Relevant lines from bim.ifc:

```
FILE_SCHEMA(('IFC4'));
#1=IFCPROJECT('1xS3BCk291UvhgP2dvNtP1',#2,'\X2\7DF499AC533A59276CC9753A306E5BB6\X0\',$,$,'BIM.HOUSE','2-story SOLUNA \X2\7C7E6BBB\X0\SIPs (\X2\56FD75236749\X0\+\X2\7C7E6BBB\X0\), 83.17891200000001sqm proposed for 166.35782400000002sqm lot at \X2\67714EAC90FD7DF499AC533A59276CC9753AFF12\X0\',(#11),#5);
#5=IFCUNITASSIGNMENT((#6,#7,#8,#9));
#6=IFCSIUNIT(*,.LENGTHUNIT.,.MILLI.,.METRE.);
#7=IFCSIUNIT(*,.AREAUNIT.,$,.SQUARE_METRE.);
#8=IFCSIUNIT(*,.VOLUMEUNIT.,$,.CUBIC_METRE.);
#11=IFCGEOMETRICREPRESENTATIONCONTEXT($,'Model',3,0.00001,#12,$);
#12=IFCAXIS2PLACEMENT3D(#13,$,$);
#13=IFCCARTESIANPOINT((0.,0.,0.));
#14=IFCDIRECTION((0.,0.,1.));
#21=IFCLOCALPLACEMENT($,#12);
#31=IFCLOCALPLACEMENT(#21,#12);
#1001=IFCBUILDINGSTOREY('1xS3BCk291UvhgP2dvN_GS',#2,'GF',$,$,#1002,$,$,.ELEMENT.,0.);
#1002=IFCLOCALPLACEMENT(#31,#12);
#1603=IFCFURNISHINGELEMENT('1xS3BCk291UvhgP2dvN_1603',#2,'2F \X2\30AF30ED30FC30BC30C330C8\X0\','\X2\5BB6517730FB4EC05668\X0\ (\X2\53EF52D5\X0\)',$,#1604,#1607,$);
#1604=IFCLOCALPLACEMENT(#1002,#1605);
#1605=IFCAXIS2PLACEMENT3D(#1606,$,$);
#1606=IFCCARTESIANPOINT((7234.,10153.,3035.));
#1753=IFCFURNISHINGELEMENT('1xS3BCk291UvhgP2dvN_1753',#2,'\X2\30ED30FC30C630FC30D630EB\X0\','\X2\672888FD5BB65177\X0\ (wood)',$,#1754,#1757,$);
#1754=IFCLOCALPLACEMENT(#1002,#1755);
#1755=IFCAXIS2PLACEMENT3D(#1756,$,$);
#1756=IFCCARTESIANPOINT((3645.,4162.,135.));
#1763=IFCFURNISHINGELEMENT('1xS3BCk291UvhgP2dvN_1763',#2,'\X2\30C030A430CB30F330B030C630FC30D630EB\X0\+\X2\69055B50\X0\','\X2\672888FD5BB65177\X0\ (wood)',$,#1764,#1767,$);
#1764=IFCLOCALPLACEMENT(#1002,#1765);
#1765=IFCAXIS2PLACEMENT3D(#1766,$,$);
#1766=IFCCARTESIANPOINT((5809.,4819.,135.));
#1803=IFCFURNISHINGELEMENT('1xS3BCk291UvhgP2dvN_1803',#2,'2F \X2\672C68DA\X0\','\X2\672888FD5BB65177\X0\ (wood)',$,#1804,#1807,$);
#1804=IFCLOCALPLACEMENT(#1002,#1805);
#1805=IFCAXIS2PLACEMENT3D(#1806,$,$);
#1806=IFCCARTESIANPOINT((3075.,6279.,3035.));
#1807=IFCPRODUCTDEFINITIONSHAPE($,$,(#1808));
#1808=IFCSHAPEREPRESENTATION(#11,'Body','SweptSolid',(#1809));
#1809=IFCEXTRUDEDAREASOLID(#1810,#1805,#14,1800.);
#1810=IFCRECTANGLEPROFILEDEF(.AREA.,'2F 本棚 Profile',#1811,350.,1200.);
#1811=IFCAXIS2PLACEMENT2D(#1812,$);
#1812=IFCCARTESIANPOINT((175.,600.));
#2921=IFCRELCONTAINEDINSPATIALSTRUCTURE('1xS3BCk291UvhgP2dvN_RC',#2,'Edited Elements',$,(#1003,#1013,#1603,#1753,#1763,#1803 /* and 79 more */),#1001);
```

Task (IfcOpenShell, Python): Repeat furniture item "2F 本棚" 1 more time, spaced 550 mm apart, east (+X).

```python
import numpy as np
import ifcopenshell
import ifcopenshell.api.geometry
import ifcopenshell.api.root
import ifcopenshell.util.element
import ifcopenshell.util.placement
import ifcopenshell.util.unit

model = ifcopenshell.open("bim.ifc")
unit_scale = ifcopenshell.util.unit.calculate_unit_scale(model)


def reuse_history(source, copy):
    """copy_class also copies each property set's owner history, people and application; keep the originals."""
    for rel in copy.IsDefinedBy:
        if rel.is_a("IfcRelDefinesByProperties") and (history := rel.RelatingPropertyDefinition.OwnerHistory):
            rel.RelatingPropertyDefinition.OwnerHistory = source.OwnerHistory
            ifcopenshell.util.element.remove_deep2(model, history)


source = model.by_guid("1xS3BCk291UvhgP2dvN_1803")
base = ifcopenshell.util.placement.get_local_placement(source.ObjectPlacement)
step = np.array([1.0, 0.0, 0.0]) * 0.55 / unit_scale

for i in range(1, 2):
    copy = ifcopenshell.api.root.copy_class(model, product=source)
    copy.Representation = ifcopenshell.util.element.copy_deep(
        model, source.Representation, exclude=["IfcGeometricRepresentationContext", "IfcRepresentationMap"]
    )
    reuse_history(source, copy)
    matrix = base.copy()
    matrix[:3, 3] += i * step
    print("added at", matrix[:3, 3].round(3) + 0.0)
    ifcopenshell.api.geometry.edit_object_placement(model, product=copy, matrix=matrix, is_si=False)

model.write("bim_updated.ifc")
```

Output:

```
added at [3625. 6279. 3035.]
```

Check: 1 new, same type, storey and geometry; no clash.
